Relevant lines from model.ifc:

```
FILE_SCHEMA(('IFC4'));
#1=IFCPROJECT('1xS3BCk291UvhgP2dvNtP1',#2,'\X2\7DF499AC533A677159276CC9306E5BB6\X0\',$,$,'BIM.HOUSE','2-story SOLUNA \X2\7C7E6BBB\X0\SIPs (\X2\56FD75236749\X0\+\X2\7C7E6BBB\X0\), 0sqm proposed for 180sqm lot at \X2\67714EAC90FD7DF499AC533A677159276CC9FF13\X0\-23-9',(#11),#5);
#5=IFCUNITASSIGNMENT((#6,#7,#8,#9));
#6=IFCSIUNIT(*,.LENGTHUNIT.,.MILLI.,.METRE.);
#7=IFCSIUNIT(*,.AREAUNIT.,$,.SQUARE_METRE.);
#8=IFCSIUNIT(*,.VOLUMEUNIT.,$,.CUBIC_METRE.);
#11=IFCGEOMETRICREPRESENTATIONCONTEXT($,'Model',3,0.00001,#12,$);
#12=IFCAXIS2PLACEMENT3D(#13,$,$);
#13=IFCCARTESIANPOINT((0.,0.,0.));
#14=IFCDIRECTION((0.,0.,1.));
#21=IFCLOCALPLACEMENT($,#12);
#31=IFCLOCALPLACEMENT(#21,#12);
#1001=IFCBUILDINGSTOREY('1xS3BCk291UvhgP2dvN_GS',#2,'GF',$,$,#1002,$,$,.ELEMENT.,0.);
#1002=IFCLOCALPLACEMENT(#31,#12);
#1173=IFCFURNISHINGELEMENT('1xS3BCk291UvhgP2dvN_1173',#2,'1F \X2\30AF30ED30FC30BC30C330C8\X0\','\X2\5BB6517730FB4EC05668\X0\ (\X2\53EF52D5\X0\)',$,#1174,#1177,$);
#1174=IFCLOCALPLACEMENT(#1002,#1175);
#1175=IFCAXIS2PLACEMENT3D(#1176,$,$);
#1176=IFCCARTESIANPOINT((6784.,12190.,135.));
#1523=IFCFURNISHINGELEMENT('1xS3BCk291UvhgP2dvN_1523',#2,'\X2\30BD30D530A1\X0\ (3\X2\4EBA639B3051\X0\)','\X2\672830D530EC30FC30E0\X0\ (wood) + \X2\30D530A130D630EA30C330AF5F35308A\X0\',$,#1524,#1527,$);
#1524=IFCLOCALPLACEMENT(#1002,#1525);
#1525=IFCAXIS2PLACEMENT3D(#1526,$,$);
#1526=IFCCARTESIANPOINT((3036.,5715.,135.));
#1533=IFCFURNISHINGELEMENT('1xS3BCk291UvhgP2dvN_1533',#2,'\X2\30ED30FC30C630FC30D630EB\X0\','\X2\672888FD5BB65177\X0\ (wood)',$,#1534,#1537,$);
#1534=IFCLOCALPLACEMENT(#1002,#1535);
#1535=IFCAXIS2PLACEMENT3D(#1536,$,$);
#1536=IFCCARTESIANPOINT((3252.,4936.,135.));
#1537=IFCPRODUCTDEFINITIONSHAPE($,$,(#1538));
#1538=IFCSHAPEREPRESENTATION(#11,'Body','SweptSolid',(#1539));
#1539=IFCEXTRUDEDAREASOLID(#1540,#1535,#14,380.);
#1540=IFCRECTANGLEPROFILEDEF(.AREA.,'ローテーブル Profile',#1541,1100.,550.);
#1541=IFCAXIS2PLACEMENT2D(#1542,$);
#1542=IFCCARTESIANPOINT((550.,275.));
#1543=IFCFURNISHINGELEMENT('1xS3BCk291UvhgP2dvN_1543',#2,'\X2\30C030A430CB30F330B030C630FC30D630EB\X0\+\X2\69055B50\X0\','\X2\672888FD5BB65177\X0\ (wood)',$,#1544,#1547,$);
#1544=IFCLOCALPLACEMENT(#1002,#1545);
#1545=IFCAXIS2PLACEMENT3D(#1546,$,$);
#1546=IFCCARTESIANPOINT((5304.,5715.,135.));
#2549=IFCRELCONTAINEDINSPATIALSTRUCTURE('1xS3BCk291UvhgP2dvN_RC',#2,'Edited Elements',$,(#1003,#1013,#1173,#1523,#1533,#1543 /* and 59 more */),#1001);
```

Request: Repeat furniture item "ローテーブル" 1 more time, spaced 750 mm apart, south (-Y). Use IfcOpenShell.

```python
import numpy as np
import ifcopenshell
import ifcopenshell.api.geometry
import ifcopenshell.api.root
import ifcopenshell.util.element
import ifcopenshell.util.placement
import ifcopenshell.util.unit

model = ifcopenshell.open("model.ifc")
unit_scale = ifcopenshell.util.unit.calculate_unit_scale(model)


def reuse_history(source, copy):
    """copy_class also copies each property set's owner history, people and application; keep the originals."""
    for rel in copy.IsDefinedBy:
        if rel.is_a("IfcRelDefinesByProperties") and (history := rel.RelatingPropertyDefinition.OwnerHistory):
            rel.RelatingPropertyDefinition.OwnerHistory = source.OwnerHistory
            ifcopenshell.util.element.remove_deep2(model, history)


source = model.by_id(1533)
base = ifcopenshell.util.placement.get_local_placement(source.ObjectPlacement)
step = np.array([0.0, -1.0, 0.0]) * 0.75 / unit_scale

for i in range(1, 2):
    copy = ifcopenshell.api.root.copy_class(model, product=source)
    copy.Representation = ifcopenshell.util.element.copy_deep(
        model, source.Representation, exclude=["IfcGeometricRepresentationContext", "IfcRepresentationMap"]
    )
    reuse_history(source, copy)
    matrix = base.copy()
    matrix[:3, 3] += i * step
    print("added at", matrix[:3, 3].round(3) + 0.0)
    ifcopenshell.api.geometry.edit_object_placement(model, product=copy, matrix=matrix, is_si=False)

model.write("model-out.ifc")
```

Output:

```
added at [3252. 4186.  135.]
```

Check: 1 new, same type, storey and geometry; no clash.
